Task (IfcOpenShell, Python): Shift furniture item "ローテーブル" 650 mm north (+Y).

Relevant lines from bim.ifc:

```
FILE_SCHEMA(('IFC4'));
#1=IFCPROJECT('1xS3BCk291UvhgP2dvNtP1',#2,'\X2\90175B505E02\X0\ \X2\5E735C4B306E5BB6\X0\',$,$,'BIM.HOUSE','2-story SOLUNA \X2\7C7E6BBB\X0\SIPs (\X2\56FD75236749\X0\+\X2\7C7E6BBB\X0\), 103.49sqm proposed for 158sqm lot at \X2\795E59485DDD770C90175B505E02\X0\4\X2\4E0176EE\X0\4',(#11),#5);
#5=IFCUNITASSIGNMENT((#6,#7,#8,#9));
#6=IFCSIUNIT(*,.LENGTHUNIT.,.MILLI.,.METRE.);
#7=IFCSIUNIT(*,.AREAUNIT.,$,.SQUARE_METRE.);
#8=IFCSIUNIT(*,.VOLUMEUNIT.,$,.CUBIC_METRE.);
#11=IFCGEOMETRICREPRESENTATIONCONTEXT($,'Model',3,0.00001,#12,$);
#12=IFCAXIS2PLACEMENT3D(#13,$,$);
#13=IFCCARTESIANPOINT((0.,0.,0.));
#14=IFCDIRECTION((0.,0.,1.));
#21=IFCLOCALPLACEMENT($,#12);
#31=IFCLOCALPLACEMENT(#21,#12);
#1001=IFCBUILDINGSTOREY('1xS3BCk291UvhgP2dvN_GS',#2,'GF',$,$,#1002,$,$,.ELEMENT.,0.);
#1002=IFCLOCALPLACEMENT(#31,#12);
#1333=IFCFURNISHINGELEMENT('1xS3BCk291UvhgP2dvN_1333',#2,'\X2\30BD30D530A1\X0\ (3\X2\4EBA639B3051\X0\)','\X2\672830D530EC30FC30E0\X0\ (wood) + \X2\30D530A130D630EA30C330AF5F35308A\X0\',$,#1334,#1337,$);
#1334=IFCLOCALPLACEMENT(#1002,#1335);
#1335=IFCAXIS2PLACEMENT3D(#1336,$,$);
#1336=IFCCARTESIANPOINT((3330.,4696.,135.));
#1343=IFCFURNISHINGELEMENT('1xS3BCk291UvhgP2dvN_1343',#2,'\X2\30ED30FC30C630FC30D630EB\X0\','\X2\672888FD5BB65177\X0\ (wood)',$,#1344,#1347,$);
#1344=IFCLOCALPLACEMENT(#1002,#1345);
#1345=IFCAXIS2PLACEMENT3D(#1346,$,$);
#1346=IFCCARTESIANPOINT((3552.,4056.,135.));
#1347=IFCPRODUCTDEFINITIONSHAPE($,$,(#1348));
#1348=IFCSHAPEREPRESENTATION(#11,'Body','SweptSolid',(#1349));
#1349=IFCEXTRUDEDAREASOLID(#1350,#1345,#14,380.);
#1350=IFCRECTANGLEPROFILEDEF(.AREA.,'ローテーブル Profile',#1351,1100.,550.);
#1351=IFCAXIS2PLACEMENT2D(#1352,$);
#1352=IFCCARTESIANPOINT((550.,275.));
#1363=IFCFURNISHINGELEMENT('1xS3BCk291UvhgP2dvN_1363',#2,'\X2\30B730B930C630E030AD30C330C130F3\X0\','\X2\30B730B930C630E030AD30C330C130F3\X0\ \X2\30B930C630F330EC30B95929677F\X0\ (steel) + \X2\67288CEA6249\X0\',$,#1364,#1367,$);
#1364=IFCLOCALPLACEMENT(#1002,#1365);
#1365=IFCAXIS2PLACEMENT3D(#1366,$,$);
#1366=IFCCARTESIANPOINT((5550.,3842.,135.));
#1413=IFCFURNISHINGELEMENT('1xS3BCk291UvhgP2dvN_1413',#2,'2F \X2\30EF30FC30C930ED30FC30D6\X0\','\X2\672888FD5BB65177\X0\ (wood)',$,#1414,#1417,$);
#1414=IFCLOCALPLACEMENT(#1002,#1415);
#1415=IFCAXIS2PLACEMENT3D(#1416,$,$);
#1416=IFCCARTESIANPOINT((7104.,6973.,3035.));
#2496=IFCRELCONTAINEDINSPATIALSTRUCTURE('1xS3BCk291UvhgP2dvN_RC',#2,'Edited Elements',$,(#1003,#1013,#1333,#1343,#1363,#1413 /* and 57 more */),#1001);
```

```python
import ifcopenshell
import ifcopenshell.api.geometry
import ifcopenshell.util.placement
import ifcopenshell.util.unit

model = ifcopenshell.open("bim.ifc")
unit_scale = ifcopenshell.util.unit.calculate_unit_scale(model)

item = model.by_guid("1xS3BCk291UvhgP2dvN_1343")
matrix = ifcopenshell.util.placement.get_local_placement(item.ObjectPlacement)
matrix[1, 3] += 0.65 / unit_scale
ifcopenshell.api.geometry.edit_object_placement(model, product=item, matrix=matrix, is_si=False)

print(ifcopenshell.util.placement.get_local_placement(item.ObjectPlacement).round(3) + 0.0)

model.write("bim-out.ifc")
```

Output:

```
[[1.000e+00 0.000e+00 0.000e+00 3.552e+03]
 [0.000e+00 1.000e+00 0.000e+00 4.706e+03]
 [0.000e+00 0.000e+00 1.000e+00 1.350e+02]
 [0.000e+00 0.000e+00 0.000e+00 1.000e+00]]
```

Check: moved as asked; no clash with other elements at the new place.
